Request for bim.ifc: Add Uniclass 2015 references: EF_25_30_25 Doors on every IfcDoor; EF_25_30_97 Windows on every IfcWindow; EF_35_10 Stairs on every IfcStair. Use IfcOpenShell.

First a look at what the model holds.

```python
import ifcopenshell

model = ifcopenshell.open("bim.ifc")
print(model.schema)
print("classifications:", [c.Name for c in model.by_type("IfcClassification")])
for ifc_class in ("IfcDoor", "IfcRoof", "IfcStair", "IfcWall", "IfcWindow"):
    print(ifc_class, len(model.by_type(ifc_class)))
```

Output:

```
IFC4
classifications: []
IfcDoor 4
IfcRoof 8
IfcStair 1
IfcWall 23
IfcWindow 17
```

```python
import ifcopenshell
import ifcopenshell.api.classification

model = ifcopenshell.open("bim.ifc")

system = ifcopenshell.api.classification.add_classification(model, classification="Uniclass 2015")

codes = {
    "IfcDoor": ("EF_25_30_25", "Doors"),
    "IfcWindow": ("EF_25_30_97", "Windows"),
    "IfcStair": ("EF_35_10", "Stairs"),
}
for ifc_class, (code, name) in codes.items():
    products = model.by_type(ifc_class)
    ifcopenshell.api.classification.add_reference(
        model, products=products, classification=system, identification=code, name=name
    )
    print(code, len(products))

model.write("bim_v2.ifc")
```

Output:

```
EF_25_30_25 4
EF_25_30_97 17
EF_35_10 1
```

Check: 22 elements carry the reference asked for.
